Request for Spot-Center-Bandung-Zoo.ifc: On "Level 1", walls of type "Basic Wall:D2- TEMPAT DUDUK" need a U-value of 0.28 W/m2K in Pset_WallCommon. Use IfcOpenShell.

First a look at what the model holds.

```python
import ifcopenshell
import ifcopenshell.util.element

model = ifcopenshell.open("Spot-Center-Bandung-Zoo.ifc")
print(model.schema)
storey = next(s for s in model.by_type("IfcBuildingStorey") if s.Name == "Level 1")
walls = [e for e in ifcopenshell.util.element.get_decomposition(storey) if e.is_a("IfcWall")]
seen = {}
for e in walls:
    element_type = ifcopenshell.util.element.get_type(e)
    key = (element_type.Name if element_type != e and element_type else None, ifcopenshell.util.element.get_pset(e, "Pset_WallCommon", "ThermalTransmittance"))
    seen[key] = seen.get(key, 0) + 1
for (name, value), count in sorted(seen.items(), key=str):
    print(count, "x", name, "|", value)
```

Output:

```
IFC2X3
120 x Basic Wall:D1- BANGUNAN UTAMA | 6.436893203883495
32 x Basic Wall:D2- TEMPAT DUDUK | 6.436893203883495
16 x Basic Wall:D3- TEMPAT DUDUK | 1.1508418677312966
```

```python
import ifcopenshell
import ifcopenshell.api.pset
import ifcopenshell.util.element

model = ifcopenshell.open("Spot-Center-Bandung-Zoo.ifc")

storey = next(s for s in model.by_type("IfcBuildingStorey") if s.Name == "Level 1")
walls = [e for e in ifcopenshell.util.element.get_decomposition(storey) if e.is_a("IfcWall")]

count = 0
for e in walls:
    element_type = ifcopenshell.util.element.get_type(e)
    if element_type in (None, e) or element_type.Name != "Basic Wall:D2- TEMPAT DUDUK":
        continue
    # add_pset returns the element's existing set when there is one.
    pset = ifcopenshell.api.pset.add_pset(model, product=e, name="Pset_WallCommon")
    ifcopenshell.api.pset.edit_pset(model, pset=pset, properties={"ThermalTransmittance": 0.28})
    count += 1

print(count, "walls updated")

model.write("Spot-Center-Bandung-Zoo_rev.ifc")
```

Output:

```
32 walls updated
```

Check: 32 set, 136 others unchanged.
